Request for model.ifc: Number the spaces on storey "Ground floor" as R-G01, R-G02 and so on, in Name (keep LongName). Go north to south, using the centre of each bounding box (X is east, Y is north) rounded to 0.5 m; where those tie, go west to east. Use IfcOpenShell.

First a look at what the model holds.

```python
import ifcopenshell
import ifcopenshell.util.element
import ifcopenshell.util.placement

model = ifcopenshell.open("model.ifc")
print(model.schema)
storey = next(s for s in model.by_type("IfcBuildingStorey") if s.Name == "Ground floor")
spaces = [e for e in ifcopenshell.util.element.get_decomposition(storey) if e.is_a("IfcSpace")]
for e in sorted(spaces, key=lambda e: e.id()):
    origin = ifcopenshell.util.placement.get_local_placement(e.ObjectPlacement)[:3, 3]
    print(e.id(), e.Name, e.LongName, origin.round(2) + 0.0, sep=" | ")
```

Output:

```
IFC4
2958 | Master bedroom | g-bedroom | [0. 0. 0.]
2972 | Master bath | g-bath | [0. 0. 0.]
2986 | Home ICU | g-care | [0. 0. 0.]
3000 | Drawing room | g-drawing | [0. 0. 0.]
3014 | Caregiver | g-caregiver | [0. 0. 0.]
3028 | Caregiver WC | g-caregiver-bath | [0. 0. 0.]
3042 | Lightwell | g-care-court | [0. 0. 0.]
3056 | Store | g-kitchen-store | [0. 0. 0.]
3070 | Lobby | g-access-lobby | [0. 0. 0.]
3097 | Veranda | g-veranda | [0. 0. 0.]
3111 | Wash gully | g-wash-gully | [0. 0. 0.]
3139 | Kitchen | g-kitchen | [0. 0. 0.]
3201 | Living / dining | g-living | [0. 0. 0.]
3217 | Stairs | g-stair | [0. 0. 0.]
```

```python
import ifcopenshell
import ifcopenshell.geom
import ifcopenshell.util.element
import ifcopenshell.util.shape

model = ifcopenshell.open("model.ifc")
settings = ifcopenshell.geom.settings()
settings.set("use-world-coords", True)


def centre(element):
    shape = ifcopenshell.geom.create_shape(settings, element)
    return ifcopenshell.util.shape.get_bbox_centroid(shape.geometry)


storey = next(s for s in model.by_type("IfcBuildingStorey") if s.Name == "Ground floor")
spaces = [e for e in ifcopenshell.util.element.get_decomposition(storey) if e.is_a("IfcSpace")]

# Insertion points can sit at a corner or the storey origin, so sort by the geometry (in metres).
centres = {e: centre(e) for e in spaces}
spaces.sort(key=lambda e: (-round(centres[e][1] / 0.5), centres[e][0]))

for i, e in enumerate(spaces, start=1):
    number = f"R-G{i:02d}"
    e.Name = number
    print(e.id(), number)

model.write("model_edited.ifc")
```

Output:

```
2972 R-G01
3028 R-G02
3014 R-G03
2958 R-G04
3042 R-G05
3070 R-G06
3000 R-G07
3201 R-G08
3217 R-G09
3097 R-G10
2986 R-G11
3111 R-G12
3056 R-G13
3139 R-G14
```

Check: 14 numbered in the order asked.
